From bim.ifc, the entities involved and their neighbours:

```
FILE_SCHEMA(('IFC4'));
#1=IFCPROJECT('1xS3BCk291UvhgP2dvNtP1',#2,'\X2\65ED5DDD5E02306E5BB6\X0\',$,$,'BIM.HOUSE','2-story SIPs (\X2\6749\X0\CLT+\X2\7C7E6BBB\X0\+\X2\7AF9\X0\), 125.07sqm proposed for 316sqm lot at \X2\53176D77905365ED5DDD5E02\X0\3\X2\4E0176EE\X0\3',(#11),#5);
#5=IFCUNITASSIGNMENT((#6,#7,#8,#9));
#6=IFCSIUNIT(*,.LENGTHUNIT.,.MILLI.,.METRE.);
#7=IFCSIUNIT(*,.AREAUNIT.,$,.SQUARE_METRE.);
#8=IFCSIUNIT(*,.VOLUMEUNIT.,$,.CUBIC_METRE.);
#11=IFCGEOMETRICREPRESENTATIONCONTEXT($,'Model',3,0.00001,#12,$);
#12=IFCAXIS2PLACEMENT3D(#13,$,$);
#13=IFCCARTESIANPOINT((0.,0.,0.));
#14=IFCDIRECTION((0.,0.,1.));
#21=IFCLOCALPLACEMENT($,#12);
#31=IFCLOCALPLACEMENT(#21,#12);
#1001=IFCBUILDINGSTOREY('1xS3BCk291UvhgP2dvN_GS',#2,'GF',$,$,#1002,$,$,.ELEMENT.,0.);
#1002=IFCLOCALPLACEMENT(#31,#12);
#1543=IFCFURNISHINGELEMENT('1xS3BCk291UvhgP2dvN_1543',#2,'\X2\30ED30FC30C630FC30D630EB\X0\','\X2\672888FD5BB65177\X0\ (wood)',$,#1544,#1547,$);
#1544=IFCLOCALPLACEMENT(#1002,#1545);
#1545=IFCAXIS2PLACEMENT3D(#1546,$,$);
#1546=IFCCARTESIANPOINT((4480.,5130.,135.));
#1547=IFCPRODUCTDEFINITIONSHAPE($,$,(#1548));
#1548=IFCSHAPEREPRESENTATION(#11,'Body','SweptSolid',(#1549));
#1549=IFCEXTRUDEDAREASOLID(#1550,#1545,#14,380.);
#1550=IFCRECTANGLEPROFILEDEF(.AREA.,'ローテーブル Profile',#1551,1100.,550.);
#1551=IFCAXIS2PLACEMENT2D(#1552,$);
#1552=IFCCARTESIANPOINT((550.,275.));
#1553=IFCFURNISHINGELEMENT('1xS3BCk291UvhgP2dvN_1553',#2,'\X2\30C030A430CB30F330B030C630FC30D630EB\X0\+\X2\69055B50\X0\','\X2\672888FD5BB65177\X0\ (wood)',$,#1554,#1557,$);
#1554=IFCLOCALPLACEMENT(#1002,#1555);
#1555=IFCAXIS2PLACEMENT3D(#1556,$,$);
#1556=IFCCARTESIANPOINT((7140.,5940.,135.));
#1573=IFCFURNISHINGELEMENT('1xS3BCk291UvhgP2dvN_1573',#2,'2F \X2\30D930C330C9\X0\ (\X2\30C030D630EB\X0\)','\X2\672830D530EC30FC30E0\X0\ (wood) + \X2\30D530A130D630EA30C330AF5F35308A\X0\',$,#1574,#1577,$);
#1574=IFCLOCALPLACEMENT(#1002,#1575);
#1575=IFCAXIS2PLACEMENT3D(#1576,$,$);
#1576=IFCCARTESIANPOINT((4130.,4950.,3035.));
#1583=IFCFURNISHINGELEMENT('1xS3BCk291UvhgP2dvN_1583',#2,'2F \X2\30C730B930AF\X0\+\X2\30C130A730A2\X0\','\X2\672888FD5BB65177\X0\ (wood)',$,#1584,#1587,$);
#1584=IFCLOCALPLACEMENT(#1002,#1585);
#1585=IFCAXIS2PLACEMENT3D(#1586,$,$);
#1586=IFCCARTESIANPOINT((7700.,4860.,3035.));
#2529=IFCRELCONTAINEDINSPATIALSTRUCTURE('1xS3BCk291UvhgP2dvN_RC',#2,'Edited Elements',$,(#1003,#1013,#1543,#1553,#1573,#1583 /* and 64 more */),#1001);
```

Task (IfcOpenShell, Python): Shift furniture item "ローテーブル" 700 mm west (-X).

```python
import ifcopenshell
import ifcopenshell.api.geometry
import ifcopenshell.util.placement

model = ifcopenshell.open("bim.ifc")

item = model.by_guid("1xS3BCk291UvhgP2dvN_1543")
matrix = ifcopenshell.util.placement.get_local_placement(item.ObjectPlacement)
matrix[0, 3] -= 700.0
ifcopenshell.api.geometry.edit_object_placement(model, product=item, matrix=matrix, is_si=False)

print(ifcopenshell.util.placement.get_local_placement(item.ObjectPlacement).round(3) + 0.0)

model.write("bim-out.ifc")
```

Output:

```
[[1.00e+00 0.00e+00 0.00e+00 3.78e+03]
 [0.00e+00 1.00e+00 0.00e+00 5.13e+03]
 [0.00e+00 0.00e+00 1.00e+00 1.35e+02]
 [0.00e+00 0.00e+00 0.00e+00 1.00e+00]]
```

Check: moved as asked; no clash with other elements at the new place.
